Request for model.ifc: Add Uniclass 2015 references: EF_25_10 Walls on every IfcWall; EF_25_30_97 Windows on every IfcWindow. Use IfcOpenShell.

First a look at what the model holds.

```python
import ifcopenshell

model = ifcopenshell.open("model.ifc")
print(model.schema)
print("classifications:", [c.Name for c in model.by_type("IfcClassification")])
for ifc_class in ("IfcDoor", "IfcRoof", "IfcStair", "IfcWall", "IfcWindow"):
    print(ifc_class, len(model.by_type(ifc_class)))
```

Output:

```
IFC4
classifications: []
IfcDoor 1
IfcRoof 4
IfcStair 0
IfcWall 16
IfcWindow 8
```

```python
import ifcopenshell
import ifcopenshell.api.classification

model = ifcopenshell.open("model.ifc")

system = ifcopenshell.api.classification.add_classification(model, classification="Uniclass 2015")

codes = {
    "IfcWall": ("EF_25_10", "Walls"),
    "IfcWindow": ("EF_25_30_97", "Windows"),
}
for ifc_class, (code, name) in codes.items():
    products = model.by_type(ifc_class)
    ifcopenshell.api.classification.add_reference(
        model, products=products, classification=system, identification=code, name=name
    )
    print(code, len(products))

model.write("model_edited.ifc")
```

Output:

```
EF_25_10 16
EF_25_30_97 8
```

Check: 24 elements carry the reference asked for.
